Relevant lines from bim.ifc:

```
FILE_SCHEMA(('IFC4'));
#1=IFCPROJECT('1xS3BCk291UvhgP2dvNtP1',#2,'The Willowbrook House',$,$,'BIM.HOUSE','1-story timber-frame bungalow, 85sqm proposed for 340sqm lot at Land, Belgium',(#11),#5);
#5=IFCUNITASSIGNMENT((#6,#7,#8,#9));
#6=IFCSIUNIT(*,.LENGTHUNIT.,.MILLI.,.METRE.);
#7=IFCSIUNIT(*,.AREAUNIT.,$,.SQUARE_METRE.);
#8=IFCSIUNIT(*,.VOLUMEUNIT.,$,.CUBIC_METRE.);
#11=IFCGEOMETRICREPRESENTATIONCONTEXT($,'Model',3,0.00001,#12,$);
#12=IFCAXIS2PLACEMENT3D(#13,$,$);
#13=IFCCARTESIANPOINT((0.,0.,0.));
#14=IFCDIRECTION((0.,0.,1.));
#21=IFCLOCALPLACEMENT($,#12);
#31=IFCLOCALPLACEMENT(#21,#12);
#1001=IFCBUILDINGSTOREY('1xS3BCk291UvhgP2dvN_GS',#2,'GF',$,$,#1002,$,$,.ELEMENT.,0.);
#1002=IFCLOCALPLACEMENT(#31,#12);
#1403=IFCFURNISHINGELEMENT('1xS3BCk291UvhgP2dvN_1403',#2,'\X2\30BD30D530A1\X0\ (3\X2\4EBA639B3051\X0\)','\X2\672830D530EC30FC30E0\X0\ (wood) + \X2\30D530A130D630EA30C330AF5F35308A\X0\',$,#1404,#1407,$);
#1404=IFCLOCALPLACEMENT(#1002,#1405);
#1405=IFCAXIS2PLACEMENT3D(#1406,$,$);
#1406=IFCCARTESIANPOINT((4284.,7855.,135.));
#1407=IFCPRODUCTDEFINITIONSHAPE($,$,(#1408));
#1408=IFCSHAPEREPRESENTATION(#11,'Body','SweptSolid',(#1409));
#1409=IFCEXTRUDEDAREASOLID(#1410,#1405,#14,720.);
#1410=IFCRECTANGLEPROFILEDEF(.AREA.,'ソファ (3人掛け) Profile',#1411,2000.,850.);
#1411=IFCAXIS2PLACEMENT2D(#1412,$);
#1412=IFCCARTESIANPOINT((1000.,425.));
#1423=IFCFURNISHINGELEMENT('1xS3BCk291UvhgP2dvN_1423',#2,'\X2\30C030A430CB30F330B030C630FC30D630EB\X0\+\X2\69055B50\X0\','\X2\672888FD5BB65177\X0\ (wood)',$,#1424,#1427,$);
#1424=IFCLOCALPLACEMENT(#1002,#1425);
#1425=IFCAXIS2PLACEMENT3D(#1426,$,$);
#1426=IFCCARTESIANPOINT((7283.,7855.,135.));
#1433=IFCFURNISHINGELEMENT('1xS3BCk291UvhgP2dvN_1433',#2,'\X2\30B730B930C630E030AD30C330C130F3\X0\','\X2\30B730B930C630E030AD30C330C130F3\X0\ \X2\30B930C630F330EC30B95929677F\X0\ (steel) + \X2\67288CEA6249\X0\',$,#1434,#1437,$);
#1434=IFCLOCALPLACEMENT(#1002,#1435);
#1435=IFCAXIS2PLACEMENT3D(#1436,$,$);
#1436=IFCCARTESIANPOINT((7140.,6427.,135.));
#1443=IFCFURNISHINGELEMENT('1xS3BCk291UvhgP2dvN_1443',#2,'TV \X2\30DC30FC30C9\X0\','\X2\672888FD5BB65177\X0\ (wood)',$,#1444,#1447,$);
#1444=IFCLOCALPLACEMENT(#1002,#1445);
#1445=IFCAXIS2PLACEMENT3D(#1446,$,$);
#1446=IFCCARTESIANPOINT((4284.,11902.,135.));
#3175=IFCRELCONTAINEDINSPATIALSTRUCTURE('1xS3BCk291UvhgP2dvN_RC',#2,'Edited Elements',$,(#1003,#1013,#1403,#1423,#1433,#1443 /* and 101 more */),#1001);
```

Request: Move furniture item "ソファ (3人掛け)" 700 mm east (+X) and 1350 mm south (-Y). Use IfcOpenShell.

```python
import ifcopenshell
import ifcopenshell.api.geometry
import ifcopenshell.util.placement
import ifcopenshell.util.unit

model = ifcopenshell.open("bim.ifc")
unit_scale = ifcopenshell.util.unit.calculate_unit_scale(model)

item = model.by_id(1403)
matrix = ifcopenshell.util.placement.get_local_placement(item.ObjectPlacement)
matrix[0, 3] += 0.7 / unit_scale
matrix[1, 3] -= 1.35 / unit_scale
ifcopenshell.api.geometry.edit_object_placement(model, product=item, matrix=matrix, is_si=False)

print(ifcopenshell.util.placement.get_local_placement(item.ObjectPlacement).round(3) + 0.0)

model.write("bim-out.ifc")
```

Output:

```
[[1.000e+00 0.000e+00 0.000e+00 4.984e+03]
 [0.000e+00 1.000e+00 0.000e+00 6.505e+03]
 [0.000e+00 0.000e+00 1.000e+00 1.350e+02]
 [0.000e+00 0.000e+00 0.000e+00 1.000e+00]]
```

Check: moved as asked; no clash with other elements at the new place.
